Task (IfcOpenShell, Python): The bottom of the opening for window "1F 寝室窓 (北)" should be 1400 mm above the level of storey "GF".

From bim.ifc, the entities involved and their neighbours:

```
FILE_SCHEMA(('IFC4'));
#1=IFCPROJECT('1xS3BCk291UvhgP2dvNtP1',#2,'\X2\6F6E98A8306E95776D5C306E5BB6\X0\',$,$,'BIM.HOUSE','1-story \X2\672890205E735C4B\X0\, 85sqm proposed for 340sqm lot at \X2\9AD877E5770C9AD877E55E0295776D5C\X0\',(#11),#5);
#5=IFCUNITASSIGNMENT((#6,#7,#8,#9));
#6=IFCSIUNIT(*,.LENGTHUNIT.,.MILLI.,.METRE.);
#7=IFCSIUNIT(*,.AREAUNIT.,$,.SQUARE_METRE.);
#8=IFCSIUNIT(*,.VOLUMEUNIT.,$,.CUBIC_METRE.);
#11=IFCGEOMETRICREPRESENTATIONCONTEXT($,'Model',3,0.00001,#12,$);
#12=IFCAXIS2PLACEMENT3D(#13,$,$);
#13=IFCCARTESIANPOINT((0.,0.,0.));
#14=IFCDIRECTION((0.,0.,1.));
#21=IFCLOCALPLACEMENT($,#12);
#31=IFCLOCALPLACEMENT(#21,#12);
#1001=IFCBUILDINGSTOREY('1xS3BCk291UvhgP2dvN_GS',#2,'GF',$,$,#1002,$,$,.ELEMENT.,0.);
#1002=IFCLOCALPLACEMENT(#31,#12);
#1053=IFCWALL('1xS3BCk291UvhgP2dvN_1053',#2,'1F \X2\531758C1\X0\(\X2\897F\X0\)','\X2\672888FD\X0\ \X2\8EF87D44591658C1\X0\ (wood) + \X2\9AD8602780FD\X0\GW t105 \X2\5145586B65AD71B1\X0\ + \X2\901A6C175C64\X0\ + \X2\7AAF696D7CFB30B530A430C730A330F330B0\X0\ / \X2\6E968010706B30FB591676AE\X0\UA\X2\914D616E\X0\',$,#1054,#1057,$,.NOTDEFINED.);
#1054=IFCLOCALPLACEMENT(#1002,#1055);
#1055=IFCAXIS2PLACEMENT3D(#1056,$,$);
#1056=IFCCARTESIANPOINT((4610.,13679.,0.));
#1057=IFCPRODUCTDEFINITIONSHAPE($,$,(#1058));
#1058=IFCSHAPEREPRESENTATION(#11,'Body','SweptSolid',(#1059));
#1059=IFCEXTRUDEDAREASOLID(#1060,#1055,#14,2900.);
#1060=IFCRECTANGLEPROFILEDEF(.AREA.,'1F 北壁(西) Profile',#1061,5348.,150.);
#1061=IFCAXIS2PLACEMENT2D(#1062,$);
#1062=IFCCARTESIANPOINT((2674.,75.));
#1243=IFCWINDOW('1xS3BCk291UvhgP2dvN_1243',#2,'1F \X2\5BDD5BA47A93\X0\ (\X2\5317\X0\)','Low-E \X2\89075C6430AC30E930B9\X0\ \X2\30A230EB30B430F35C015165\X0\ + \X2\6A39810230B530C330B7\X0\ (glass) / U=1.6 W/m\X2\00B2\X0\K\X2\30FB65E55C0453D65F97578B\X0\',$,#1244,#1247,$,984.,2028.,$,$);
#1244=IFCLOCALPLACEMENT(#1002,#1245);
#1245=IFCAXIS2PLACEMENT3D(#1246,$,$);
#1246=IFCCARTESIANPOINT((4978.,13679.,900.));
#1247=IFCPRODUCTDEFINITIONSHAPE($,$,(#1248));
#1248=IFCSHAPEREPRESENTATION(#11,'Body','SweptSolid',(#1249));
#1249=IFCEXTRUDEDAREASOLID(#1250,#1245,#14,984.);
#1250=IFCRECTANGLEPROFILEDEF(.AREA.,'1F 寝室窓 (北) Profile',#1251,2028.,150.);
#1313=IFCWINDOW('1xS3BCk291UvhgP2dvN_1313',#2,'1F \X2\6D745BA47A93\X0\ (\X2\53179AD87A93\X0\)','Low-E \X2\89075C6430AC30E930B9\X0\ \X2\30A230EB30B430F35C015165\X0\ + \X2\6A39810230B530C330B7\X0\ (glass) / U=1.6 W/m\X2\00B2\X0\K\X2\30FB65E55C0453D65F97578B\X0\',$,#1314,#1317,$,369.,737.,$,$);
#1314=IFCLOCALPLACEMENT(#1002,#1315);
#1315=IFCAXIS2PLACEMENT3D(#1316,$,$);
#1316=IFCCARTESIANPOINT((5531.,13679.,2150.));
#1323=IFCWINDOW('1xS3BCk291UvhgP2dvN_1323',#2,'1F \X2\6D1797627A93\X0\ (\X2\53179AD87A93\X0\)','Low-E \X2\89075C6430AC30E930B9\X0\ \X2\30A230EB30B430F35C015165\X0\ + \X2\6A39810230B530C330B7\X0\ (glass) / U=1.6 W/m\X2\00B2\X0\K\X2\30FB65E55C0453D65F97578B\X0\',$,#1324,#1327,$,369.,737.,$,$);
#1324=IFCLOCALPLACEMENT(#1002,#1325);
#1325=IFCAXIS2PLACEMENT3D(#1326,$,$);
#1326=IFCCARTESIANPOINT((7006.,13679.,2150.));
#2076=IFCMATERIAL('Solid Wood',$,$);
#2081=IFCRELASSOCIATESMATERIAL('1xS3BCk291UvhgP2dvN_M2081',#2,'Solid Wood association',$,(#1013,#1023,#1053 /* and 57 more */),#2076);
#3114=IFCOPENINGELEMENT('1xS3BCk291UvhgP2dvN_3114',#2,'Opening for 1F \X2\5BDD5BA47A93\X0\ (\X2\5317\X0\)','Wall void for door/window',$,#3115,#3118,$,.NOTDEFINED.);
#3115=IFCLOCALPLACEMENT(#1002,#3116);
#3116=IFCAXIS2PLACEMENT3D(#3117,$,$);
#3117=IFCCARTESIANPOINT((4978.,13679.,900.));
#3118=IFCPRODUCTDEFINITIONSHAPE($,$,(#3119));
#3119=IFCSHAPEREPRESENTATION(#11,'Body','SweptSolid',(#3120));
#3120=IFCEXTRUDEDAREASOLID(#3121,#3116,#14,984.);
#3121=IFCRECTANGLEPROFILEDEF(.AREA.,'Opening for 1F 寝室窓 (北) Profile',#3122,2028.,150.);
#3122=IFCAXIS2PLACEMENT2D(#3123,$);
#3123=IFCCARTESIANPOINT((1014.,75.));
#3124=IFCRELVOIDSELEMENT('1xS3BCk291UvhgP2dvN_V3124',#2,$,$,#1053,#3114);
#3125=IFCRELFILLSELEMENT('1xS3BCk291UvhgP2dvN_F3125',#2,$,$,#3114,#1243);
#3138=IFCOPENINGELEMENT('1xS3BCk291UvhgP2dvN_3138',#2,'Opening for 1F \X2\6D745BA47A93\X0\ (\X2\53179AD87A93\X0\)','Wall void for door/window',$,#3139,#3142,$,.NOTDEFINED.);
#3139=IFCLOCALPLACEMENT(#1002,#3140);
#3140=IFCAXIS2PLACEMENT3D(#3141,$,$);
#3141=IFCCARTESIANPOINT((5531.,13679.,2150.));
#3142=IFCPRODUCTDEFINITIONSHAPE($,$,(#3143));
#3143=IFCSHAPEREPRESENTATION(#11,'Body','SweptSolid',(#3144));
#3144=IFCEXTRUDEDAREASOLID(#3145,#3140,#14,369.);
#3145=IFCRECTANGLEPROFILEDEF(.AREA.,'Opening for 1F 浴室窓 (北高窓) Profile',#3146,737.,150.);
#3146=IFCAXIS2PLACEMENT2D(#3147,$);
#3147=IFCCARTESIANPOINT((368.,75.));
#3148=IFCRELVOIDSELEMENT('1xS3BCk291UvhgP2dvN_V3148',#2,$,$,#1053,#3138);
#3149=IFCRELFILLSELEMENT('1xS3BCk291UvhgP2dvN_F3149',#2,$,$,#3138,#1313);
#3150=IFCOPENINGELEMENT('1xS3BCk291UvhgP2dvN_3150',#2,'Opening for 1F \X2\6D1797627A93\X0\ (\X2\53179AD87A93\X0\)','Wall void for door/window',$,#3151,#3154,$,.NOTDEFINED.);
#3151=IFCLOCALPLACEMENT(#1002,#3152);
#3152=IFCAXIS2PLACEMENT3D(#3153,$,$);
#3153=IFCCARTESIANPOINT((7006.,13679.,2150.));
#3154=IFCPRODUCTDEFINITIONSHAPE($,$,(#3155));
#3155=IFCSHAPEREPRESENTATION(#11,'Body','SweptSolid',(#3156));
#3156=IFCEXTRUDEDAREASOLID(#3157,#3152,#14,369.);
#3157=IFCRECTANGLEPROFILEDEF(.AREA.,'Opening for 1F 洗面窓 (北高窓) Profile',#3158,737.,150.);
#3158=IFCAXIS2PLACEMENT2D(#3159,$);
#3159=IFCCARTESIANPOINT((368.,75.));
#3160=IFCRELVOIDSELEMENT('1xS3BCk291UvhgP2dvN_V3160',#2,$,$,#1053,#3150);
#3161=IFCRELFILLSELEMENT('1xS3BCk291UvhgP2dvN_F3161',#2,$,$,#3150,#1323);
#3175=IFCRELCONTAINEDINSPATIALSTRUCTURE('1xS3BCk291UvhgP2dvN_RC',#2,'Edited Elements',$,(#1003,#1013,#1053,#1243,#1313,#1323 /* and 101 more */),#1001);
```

```python
import numpy as np
import ifcopenshell
import ifcopenshell.api.geometry
import ifcopenshell.geom
import ifcopenshell.util.element
import ifcopenshell.util.placement
import ifcopenshell.util.shape
import ifcopenshell.util.unit

model = ifcopenshell.open("bim.ifc")
unit_scale = ifcopenshell.util.unit.calculate_unit_scale(model)

window = model.by_guid("1xS3BCk291UvhgP2dvN_1243")
opening = window.FillsVoids[0].RelatingOpeningElement
storey = ifcopenshell.util.element.get_container(window, ifc_class="IfcBuildingStorey")
level = ifcopenshell.util.placement.get_local_placement(storey.ObjectPlacement)[2, 3]

# The opening's origin need not be at the sill, so measure its lowest point.
shape = ifcopenshell.geom.create_shape(ifcopenshell.geom.settings(), opening)
bottom = ifcopenshell.util.shape.get_shape_bottom_elevation(shape, shape.geometry) / unit_scale
dz = level + 1400.0 - bottom

shift = np.array([0.0, 0.0, dz])
# The window is not placed relative to its opening, so move both.
for product in (opening, window):
    matrix = ifcopenshell.util.placement.get_local_placement(product.ObjectPlacement)
    matrix[:3, 3] += shift
    ifcopenshell.api.geometry.edit_object_placement(model, product=product, matrix=matrix, is_si=False)

print(f"moved by {dz * unit_scale:+.3f} m")

model.write("bim_v2.ifc")
```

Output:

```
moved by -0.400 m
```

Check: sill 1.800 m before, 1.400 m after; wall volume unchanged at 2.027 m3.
